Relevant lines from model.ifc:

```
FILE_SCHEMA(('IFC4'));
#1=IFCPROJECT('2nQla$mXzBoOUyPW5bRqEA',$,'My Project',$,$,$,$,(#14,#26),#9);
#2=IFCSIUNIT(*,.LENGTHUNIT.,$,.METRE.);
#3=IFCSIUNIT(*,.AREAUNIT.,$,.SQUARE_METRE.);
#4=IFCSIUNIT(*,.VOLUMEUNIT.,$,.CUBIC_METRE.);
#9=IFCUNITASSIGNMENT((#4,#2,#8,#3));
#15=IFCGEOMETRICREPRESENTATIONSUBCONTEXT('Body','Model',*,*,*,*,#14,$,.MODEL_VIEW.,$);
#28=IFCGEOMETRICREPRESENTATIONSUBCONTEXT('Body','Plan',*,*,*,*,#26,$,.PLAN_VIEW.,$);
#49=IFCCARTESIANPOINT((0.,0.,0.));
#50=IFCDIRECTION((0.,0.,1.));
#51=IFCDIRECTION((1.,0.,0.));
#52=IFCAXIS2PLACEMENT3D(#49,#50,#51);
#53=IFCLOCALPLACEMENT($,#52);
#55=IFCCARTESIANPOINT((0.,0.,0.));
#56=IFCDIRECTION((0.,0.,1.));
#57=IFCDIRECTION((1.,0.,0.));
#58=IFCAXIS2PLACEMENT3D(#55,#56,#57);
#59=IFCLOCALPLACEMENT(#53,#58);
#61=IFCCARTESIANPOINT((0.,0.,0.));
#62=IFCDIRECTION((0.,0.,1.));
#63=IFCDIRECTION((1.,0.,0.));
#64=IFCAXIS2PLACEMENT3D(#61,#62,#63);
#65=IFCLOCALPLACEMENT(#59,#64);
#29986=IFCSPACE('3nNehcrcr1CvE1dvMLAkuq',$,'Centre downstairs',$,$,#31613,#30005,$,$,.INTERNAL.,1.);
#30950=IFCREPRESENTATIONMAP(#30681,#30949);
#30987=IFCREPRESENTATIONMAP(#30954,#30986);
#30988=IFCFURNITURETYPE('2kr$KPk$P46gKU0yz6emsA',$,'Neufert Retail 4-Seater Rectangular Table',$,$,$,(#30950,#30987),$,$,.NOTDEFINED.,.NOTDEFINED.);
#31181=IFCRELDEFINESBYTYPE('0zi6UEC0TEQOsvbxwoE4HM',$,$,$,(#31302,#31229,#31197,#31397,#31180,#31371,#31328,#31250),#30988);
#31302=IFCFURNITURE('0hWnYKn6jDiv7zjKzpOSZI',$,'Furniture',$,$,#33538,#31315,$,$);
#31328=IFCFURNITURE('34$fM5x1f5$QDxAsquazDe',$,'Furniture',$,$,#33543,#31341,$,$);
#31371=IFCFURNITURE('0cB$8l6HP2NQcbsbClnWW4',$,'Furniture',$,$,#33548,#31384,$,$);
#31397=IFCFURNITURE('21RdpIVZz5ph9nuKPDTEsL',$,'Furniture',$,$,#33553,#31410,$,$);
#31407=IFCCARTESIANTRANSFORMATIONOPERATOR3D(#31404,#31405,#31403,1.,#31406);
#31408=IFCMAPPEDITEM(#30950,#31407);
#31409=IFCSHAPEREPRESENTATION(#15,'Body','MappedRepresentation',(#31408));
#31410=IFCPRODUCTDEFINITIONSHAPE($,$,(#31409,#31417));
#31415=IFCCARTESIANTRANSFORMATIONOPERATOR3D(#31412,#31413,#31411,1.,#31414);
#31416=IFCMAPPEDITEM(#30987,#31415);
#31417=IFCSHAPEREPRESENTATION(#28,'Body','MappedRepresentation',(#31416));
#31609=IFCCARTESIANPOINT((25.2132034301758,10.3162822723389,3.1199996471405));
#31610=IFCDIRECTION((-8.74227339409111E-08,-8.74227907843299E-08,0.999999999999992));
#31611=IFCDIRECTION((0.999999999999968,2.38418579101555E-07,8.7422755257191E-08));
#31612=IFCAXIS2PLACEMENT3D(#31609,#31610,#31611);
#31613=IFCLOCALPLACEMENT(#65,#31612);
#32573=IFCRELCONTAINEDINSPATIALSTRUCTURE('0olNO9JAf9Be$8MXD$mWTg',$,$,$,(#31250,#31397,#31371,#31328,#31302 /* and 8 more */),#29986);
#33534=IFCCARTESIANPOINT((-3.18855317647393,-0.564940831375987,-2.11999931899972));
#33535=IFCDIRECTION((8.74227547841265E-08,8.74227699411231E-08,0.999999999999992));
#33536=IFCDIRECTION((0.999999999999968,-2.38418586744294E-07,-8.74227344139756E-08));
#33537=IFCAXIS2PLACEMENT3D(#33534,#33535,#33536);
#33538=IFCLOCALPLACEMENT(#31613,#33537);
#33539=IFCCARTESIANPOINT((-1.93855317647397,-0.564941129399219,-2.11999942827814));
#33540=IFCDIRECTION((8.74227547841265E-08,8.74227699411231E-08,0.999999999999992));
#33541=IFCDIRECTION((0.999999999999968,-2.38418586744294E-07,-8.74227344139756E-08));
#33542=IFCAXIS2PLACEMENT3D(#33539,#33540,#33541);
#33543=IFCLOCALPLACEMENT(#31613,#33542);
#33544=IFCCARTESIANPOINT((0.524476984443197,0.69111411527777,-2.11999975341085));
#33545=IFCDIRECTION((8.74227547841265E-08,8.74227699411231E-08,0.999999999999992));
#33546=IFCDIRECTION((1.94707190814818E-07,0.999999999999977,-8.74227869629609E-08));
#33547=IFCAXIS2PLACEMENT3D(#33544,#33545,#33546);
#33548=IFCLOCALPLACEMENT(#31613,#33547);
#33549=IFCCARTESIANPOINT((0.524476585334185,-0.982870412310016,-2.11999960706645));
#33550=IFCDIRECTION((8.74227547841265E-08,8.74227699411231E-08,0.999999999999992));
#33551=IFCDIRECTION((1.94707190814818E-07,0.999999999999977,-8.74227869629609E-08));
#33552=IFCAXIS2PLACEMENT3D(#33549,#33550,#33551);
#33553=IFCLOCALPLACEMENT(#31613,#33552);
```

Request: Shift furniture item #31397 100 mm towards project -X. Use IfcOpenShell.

```python
import ifcopenshell
import ifcopenshell.api.geometry
import ifcopenshell.util.placement

model = ifcopenshell.open("model.ifc")

item = model.by_id(31397)
matrix = ifcopenshell.util.placement.get_local_placement(item.ObjectPlacement)
matrix[0, 3] -= 0.1
ifcopenshell.api.geometry.edit_object_placement(model, product=item, matrix=matrix, is_si=False)

print(ifcopenshell.util.placement.get_local_placement(item.ObjectPlacement).round(3) + 0.0)

model.write("model-out.ifc")
```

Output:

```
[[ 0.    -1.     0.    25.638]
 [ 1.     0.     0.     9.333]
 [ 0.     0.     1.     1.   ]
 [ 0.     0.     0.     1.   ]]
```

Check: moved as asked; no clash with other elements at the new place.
